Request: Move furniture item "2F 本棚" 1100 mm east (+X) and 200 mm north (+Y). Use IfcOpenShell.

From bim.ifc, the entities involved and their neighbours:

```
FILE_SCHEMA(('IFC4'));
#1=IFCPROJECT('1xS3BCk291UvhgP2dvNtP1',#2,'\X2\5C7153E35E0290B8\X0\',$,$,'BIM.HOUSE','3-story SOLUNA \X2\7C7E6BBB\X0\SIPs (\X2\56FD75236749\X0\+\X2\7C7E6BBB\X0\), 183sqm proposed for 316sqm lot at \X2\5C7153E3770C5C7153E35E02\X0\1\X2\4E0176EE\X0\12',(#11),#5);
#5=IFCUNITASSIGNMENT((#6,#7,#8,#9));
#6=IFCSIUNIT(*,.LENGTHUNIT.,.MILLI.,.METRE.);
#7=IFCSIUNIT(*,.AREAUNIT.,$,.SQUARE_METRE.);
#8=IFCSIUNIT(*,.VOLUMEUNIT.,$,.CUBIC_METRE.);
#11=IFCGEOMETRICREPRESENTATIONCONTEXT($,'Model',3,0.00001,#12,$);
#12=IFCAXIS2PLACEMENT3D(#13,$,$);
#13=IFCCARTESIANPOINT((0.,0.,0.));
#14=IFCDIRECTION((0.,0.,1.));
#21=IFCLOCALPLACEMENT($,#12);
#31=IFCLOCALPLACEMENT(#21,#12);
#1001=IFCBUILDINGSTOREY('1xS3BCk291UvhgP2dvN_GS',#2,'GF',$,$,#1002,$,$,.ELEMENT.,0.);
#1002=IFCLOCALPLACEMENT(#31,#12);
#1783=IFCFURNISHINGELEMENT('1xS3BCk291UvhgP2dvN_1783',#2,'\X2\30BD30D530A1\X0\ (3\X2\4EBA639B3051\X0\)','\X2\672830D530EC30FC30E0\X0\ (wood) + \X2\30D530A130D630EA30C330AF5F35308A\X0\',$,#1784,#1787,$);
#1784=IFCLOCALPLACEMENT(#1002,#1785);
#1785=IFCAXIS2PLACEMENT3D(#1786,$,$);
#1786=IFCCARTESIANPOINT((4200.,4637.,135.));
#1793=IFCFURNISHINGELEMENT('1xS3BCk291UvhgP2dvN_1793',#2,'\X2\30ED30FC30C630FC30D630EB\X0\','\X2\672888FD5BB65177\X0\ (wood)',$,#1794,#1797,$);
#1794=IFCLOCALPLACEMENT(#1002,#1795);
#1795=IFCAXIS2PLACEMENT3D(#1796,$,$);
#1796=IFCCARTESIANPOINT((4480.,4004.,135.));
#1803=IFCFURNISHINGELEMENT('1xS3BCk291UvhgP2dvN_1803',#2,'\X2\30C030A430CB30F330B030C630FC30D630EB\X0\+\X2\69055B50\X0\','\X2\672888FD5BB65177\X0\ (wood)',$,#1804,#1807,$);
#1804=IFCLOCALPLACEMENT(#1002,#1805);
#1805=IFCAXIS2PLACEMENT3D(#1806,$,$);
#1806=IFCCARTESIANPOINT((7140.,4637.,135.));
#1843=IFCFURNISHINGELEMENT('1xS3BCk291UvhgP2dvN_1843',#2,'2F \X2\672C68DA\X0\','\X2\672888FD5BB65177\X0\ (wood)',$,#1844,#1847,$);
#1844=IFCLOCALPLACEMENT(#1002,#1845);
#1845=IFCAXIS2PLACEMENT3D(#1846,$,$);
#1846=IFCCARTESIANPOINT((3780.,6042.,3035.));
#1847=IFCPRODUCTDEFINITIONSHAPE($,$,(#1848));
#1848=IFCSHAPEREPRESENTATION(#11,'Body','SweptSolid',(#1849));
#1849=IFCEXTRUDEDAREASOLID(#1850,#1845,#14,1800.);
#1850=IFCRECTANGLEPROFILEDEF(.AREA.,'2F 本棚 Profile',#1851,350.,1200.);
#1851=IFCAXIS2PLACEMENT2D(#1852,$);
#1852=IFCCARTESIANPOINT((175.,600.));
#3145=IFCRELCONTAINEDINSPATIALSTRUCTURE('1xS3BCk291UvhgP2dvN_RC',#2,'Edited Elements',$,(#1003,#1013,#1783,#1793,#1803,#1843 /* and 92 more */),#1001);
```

```python
import ifcopenshell
import ifcopenshell.api.geometry
import ifcopenshell.util.placement
import ifcopenshell.util.unit

model = ifcopenshell.open("bim.ifc")
unit_scale = ifcopenshell.util.unit.calculate_unit_scale(model)

item = model.by_guid("1xS3BCk291UvhgP2dvN_1843")
matrix = ifcopenshell.util.placement.get_local_placement(item.ObjectPlacement)
matrix[0, 3] += 1.1 / unit_scale
matrix[1, 3] += 0.2 / unit_scale
ifcopenshell.api.geometry.edit_object_placement(model, product=item, matrix=matrix, is_si=False)

print(ifcopenshell.util.placement.get_local_placement(item.ObjectPlacement).round(3) + 0.0)

model.write("bim_edited.ifc")
```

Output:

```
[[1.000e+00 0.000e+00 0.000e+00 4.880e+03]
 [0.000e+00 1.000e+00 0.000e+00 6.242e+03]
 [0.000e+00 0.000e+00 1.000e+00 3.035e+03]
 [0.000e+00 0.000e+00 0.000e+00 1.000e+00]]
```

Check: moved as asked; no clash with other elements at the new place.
